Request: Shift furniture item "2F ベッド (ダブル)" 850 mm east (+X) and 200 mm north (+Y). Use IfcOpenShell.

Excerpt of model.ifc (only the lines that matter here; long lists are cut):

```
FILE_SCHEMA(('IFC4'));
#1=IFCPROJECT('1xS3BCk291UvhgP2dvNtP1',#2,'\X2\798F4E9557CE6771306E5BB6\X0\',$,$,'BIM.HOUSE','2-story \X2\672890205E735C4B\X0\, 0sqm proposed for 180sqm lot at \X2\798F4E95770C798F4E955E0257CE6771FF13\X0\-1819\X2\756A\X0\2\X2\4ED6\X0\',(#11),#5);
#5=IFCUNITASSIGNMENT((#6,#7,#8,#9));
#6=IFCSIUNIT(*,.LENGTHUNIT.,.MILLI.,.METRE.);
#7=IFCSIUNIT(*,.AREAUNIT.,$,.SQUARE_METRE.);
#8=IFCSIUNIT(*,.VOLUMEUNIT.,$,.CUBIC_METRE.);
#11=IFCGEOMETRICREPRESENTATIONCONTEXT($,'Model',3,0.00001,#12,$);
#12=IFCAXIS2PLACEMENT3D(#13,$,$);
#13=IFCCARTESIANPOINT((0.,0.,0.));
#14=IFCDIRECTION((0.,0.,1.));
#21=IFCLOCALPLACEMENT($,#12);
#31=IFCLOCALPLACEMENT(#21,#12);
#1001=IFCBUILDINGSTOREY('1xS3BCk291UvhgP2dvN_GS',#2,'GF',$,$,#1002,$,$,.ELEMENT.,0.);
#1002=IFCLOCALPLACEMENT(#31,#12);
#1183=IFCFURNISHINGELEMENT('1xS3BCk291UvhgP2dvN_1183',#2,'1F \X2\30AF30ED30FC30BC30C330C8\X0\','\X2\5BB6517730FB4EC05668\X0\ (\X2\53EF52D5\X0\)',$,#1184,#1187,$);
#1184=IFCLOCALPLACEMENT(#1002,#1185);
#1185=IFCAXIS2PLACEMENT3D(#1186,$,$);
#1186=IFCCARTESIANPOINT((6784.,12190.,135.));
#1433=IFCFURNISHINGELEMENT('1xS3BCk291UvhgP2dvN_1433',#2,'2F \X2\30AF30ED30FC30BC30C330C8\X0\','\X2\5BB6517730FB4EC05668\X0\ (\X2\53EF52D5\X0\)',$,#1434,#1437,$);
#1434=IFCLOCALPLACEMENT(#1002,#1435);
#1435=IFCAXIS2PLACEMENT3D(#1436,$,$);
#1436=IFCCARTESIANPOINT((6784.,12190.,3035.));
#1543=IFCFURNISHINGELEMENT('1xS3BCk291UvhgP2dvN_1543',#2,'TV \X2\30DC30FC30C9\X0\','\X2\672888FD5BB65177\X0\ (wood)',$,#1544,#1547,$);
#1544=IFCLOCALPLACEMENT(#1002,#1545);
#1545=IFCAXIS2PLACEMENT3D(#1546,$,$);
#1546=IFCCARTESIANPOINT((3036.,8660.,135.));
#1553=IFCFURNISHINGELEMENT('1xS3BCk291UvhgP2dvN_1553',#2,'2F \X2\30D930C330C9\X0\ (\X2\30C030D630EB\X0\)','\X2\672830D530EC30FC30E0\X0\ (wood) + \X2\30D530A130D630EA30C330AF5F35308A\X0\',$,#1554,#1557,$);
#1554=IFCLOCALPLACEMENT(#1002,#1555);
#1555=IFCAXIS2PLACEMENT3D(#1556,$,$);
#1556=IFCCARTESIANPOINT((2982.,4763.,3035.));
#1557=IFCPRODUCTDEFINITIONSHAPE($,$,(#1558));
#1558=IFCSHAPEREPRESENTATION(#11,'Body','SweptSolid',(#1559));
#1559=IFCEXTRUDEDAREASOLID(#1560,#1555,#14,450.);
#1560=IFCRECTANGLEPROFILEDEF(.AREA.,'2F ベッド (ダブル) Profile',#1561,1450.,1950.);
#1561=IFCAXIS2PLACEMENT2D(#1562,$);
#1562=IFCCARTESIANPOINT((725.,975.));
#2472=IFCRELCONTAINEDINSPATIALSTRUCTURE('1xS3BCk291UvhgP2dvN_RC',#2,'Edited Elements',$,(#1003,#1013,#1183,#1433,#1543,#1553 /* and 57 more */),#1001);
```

```python
import ifcopenshell
import ifcopenshell.api.geometry
import ifcopenshell.util.placement

model = ifcopenshell.open("model.ifc")

item = model.by_guid("1xS3BCk291UvhgP2dvN_1553")
matrix = ifcopenshell.util.placement.get_local_placement(item.ObjectPlacement)
matrix[0, 3] += 850.0
matrix[1, 3] += 200.0
ifcopenshell.api.geometry.edit_object_placement(model, product=item, matrix=matrix, is_si=False)

print(ifcopenshell.util.placement.get_local_placement(item.ObjectPlacement).round(3) + 0.0)

model.write("model-out.ifc")
```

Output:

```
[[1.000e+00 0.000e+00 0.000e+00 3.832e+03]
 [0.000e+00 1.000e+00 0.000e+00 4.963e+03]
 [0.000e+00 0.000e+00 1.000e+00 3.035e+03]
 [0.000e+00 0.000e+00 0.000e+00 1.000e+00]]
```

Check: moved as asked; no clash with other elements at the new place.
